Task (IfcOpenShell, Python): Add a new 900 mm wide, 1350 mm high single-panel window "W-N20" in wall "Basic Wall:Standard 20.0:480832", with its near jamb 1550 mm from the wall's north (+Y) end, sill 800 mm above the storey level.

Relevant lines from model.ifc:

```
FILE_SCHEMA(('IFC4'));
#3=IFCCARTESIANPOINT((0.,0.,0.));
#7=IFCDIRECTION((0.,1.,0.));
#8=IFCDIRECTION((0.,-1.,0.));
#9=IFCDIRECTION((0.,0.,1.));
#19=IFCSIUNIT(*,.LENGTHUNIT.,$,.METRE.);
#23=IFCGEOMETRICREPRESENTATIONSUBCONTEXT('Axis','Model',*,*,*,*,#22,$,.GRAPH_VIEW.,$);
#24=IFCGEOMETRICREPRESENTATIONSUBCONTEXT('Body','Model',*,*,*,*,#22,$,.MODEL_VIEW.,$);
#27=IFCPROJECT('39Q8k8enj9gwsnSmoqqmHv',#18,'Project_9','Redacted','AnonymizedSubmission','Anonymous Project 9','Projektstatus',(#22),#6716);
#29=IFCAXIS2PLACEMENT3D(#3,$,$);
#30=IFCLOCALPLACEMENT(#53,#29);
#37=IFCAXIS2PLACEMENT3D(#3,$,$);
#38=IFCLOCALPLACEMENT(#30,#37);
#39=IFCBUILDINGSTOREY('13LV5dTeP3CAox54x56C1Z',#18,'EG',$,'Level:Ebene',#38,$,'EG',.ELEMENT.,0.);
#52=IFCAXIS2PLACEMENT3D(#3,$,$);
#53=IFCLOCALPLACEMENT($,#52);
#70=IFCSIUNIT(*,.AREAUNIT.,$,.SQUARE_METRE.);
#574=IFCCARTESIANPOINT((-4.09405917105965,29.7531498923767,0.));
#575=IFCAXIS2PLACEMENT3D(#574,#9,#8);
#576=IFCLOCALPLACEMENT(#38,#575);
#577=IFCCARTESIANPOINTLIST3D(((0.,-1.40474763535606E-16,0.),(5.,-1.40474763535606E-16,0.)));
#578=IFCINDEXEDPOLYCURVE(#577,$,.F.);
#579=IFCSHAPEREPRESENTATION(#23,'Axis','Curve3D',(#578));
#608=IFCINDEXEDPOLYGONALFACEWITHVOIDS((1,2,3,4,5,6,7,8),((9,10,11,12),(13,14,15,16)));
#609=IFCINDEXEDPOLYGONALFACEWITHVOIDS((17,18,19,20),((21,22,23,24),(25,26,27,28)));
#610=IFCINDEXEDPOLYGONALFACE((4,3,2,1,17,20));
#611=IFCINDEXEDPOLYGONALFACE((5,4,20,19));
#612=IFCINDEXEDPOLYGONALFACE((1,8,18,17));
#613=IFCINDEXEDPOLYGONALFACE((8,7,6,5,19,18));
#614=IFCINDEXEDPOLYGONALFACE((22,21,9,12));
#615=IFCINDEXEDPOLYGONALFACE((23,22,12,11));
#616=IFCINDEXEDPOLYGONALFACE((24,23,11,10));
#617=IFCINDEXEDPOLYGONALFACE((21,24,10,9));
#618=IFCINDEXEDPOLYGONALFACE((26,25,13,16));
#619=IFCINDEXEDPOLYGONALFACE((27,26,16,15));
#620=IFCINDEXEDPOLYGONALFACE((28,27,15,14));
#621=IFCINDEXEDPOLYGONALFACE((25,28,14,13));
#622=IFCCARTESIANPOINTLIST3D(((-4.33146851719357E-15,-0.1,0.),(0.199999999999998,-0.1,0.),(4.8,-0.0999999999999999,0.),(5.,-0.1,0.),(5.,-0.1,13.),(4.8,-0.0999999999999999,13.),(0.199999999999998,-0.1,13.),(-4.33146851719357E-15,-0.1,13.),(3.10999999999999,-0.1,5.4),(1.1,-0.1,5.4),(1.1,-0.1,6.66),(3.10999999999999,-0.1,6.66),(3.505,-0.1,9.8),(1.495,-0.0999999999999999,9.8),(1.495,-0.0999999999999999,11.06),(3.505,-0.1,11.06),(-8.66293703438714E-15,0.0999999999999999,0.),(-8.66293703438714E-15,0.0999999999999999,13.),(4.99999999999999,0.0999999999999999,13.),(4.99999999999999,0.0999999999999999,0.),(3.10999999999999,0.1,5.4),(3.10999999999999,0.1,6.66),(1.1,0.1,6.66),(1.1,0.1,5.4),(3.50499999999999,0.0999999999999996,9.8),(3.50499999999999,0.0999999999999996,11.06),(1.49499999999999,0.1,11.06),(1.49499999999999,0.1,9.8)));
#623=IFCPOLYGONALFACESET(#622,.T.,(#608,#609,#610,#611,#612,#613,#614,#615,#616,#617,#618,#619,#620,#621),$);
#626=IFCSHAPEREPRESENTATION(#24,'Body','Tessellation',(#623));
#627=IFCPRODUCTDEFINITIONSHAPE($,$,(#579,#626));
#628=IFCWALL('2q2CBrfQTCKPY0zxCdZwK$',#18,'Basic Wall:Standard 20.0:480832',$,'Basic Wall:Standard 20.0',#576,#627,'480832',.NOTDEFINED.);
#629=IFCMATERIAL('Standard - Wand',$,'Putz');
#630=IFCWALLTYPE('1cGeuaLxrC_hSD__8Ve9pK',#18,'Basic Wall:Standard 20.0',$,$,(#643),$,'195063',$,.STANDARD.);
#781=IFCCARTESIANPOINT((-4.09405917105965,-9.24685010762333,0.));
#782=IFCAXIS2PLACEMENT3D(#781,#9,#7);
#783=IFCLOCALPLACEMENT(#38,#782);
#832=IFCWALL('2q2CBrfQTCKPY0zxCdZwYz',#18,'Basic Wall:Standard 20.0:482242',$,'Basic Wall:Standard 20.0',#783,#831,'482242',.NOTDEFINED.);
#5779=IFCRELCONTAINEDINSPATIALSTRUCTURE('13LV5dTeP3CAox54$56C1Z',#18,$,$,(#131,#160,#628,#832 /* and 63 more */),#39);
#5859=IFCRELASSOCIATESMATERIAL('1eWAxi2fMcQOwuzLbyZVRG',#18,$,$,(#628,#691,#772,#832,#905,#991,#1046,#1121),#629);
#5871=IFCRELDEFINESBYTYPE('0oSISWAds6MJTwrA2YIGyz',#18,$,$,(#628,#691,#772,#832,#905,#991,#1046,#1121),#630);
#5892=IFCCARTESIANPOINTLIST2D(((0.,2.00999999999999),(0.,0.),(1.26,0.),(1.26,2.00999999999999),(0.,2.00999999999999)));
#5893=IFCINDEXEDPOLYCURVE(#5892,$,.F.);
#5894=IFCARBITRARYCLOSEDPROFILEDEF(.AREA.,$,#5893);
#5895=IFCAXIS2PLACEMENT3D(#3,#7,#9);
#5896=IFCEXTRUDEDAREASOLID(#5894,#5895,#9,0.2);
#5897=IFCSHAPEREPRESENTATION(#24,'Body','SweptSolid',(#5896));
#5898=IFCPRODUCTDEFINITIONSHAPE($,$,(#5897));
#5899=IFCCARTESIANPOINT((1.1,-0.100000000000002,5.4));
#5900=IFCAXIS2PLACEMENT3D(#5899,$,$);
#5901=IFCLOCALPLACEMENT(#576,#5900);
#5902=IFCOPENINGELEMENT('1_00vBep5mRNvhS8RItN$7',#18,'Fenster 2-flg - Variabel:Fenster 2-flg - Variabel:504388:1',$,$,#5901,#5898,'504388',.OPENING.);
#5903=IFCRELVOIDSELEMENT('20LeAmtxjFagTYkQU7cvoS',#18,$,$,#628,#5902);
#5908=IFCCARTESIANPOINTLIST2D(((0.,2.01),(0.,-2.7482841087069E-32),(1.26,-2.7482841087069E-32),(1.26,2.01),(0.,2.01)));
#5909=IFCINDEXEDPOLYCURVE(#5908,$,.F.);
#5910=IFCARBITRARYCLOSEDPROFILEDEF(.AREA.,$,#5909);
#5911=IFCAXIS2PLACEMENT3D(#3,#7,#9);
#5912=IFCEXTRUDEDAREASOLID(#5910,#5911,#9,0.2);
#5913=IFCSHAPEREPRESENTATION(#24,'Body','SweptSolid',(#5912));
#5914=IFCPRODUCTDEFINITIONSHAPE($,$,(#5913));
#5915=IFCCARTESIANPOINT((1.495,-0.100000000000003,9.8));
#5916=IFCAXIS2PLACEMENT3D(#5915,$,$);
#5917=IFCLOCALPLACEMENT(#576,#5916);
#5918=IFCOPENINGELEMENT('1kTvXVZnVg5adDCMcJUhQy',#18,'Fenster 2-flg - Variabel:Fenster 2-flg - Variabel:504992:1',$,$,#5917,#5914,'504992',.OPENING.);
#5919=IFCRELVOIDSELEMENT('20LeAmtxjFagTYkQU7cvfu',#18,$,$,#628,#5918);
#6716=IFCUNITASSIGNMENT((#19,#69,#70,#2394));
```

```python
import numpy as np
import ifcopenshell
import ifcopenshell.api.feature
import ifcopenshell.api.geometry
import ifcopenshell.api.root
import ifcopenshell.api.spatial
import ifcopenshell.geom
import ifcopenshell.util.element
import ifcopenshell.util.placement
import ifcopenshell.util.representation
import ifcopenshell.util.shape
import ifcopenshell.util.unit

model = ifcopenshell.open("model.ifc")
unit_scale = ifcopenshell.util.unit.calculate_unit_scale(model)
settings = ifcopenshell.geom.settings()


def volume(element):
    """Net volume in cubic metres, openings subtracted."""
    shape = ifcopenshell.geom.create_shape(settings, element)
    return ifcopenshell.util.shape.get_volume(shape.geometry)


wall = model.by_id(628)
storey = ifcopenshell.util.element.get_container(wall, ifc_class="IfcBuildingStorey")
context = ifcopenshell.util.representation.get_context(model, "Model", "Body", "MODEL_VIEW")
before = volume(wall)

width, height, from_end, sill = 0.9, 1.35, 1.55, 0.8  # metres

# The wall runs along its own X axis, and the end named is its -X end.
wall_shape = ifcopenshell.geom.create_shape(settings, wall)
x, y, z = ifcopenshell.util.shape.get_vertices(wall_shape.geometry).T
start = x.min() + from_end
face, thickness = float(y.min()), float(y.max() - y.min())
wall_matrix = ifcopenshell.util.placement.get_local_placement(wall.ObjectPlacement)
level = ifcopenshell.util.placement.get_local_placement(storey.ObjectPlacement)[2, 3]


def in_wall(x, y):
    """Placement at x, y metres in the wall's axes, at sill height."""
    matrix = wall_matrix.copy()
    matrix[:, 3] = wall_matrix @ np.array([x / unit_scale, y / unit_scale, 0.0, 1.0])
    matrix[2, 3] = level + sill / unit_scale
    return matrix


# Opening: a box that overshoots both wall faces by 50 mm.
opening = ifcopenshell.api.root.create_entity(model, ifc_class="IfcOpeningElement", predefined_type="OPENING")
box = ifcopenshell.api.geometry.add_wall_representation(
    model, context=context, length=width, height=height, thickness=thickness + 0.1
)
ifcopenshell.api.geometry.assign_representation(model, product=opening, representation=box)
ifcopenshell.api.geometry.edit_object_placement(model, product=opening, matrix=in_wall(start, face - 0.05), is_si=False)
ifcopenshell.api.feature.add_feature(model, feature=opening, element=wall)

window = ifcopenshell.api.root.create_entity(model, ifc_class="IfcWindow", name="W-N20", predefined_type="WINDOW")
window.OverallWidth, window.OverallHeight = width / unit_scale, height / unit_scale
window.PartitioningType = "SINGLE_PANEL"
body = ifcopenshell.api.geometry.add_window_representation(
    model,
    context=context,
    overall_width=window.OverallWidth,
    overall_height=window.OverallHeight,
    partition_type="SINGLE_PANEL",
)
ifcopenshell.api.geometry.assign_representation(model, product=window, representation=body)
ifcopenshell.api.spatial.assign_container(model, products=[window], relating_structure=storey)
ifcopenshell.api.feature.add_filling(model, opening=opening, element=window)

# Centre the window in the wall's thickness.
ifcopenshell.api.geometry.edit_object_placement(model, product=window, matrix=in_wall(start, face), is_si=False)
window_shape = ifcopenshell.geom.create_shape(settings, window)
depth = ifcopenshell.util.shape.get_vertices(window_shape.geometry)[:, 1]
offset = face + thickness / 2 - (depth.min() + depth.max()) / 2
ifcopenshell.api.geometry.edit_object_placement(model, product=window, matrix=in_wall(start, offset), is_si=False)

after = volume(wall)

print(f"wall volume {before:.3f} -> {after:.3f} m3")

model.write("model_v2.ifc")
```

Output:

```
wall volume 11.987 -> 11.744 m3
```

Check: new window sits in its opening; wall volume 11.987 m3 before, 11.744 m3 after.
